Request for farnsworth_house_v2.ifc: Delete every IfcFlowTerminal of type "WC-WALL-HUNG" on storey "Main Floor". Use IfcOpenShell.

First a look at what the model holds.

```python
import ifcopenshell
import ifcopenshell.util.element

model = ifcopenshell.open("farnsworth_house_v2.ifc")
print(model.schema)
storey = next(s for s in model.by_type("IfcBuildingStorey") if s.Name == "Main Floor")
terminals = [e for e in ifcopenshell.util.element.get_decomposition(storey) if e.is_a("IfcFlowTerminal")]
seen = {}
for e in terminals:
    element_type = ifcopenshell.util.element.get_type(e)
    name = element_type.Name if element_type not in (None, e) else None
    seen[name] = seen.get(name, 0) + 1
for name, count in sorted(seen.items(), key=str):
    print(count, "x", name)
```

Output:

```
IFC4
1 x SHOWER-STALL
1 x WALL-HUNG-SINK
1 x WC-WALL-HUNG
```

```python
import ifcopenshell
import ifcopenshell.api.root
import ifcopenshell.util.element

model = ifcopenshell.open("farnsworth_house_v2.ifc")

storey = next(s for s in model.by_type("IfcBuildingStorey") if s.Name == "Main Floor")
terminals = [e for e in ifcopenshell.util.element.get_decomposition(storey) if e.is_a("IfcFlowTerminal")]
targets = [e for e in terminals if (t := ifcopenshell.util.element.get_type(e)) not in (None, e) and t.Name == "WC-WALL-HUNG"]

for e in targets:
    ifcopenshell.api.root.remove_product(model, product=e)
print(len(targets), "removed")

model.write("farnsworth_house_v2_rev.ifc")
```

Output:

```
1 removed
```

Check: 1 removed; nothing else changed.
